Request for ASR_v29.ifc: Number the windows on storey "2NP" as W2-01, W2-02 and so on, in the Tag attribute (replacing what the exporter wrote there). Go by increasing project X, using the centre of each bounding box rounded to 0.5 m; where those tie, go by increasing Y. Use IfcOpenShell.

First a look at what the model holds.

```python
import ifcopenshell
import ifcopenshell.util.element
import ifcopenshell.util.placement

model = ifcopenshell.open("ASR_v29.ifc")
print(model.schema)
storey = next(s for s in model.by_type("IfcBuildingStorey") if s.Name == "2NP")
windows = [e for e in ifcopenshell.util.element.get_decomposition(storey) if e.is_a("IfcWindow")]
for e in sorted(windows, key=lambda e: e.id()):
    origin = ifcopenshell.util.placement.get_local_placement(e.ObjectPlacement)[:3, 3]
    print(e.id(), e.Tag, e.Name, origin.round(2) + 0.0, sep=" | ")
```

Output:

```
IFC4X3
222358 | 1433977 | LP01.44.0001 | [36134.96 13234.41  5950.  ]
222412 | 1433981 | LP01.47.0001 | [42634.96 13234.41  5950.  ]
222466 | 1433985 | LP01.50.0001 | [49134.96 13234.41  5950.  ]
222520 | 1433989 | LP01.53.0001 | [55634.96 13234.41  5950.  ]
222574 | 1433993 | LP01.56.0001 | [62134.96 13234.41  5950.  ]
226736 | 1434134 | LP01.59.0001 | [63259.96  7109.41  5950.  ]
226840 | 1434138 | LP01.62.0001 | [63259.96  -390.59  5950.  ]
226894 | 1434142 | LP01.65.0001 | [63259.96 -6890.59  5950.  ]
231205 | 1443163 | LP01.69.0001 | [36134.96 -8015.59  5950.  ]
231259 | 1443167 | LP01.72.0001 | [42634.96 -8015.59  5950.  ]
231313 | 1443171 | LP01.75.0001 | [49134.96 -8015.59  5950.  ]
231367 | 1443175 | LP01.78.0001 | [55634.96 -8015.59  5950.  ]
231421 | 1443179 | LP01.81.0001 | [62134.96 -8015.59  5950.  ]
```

```python
import ifcopenshell
import ifcopenshell.geom
import ifcopenshell.util.element
import ifcopenshell.util.shape

model = ifcopenshell.open("ASR_v29.ifc")
settings = ifcopenshell.geom.settings()
settings.set("use-world-coords", True)


def centre(element):
    shape = ifcopenshell.geom.create_shape(settings, element)
    return ifcopenshell.util.shape.get_bbox_centroid(shape.geometry)


storey = next(s for s in model.by_type("IfcBuildingStorey") if s.Name == "2NP")
windows = [e for e in ifcopenshell.util.element.get_decomposition(storey) if e.is_a("IfcWindow")]

# Insertion points can sit at a corner or the storey origin, so sort by the geometry (in metres).
centres = {e: centre(e) for e in windows}
windows.sort(key=lambda e: (round(centres[e][0] / 0.5), centres[e][1]))

for i, e in enumerate(windows, start=1):
    number = f"W2-{i:02d}"
    e.Tag = number
    print(e.id(), number)

model.write("ASR_v29-out.ifc")
```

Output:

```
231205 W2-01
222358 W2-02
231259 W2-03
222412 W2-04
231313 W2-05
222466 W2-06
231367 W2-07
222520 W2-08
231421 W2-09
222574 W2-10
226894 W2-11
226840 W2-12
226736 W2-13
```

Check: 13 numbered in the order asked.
